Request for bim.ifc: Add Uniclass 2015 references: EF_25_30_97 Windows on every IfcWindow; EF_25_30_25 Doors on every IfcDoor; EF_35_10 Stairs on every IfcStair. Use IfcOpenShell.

First a look at what the model holds.

```python
import ifcopenshell

model = ifcopenshell.open("bim.ifc")
print(model.schema)
print("classifications:", [c.Name for c in model.by_type("IfcClassification")])
for ifc_class in ("IfcDoor", "IfcRoof", "IfcStair", "IfcWall", "IfcWindow"):
    print(ifc_class, len(model.by_type(ifc_class)))
```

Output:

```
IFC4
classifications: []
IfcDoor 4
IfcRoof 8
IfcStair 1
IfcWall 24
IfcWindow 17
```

```python
import ifcopenshell
import ifcopenshell.api.classification

model = ifcopenshell.open("bim.ifc")

system = ifcopenshell.api.classification.add_classification(model, classification="Uniclass 2015")

codes = {
    "IfcWindow": ("EF_25_30_97", "Windows"),
    "IfcDoor": ("EF_25_30_25", "Doors"),
    "IfcStair": ("EF_35_10", "Stairs"),
}
for ifc_class, (code, name) in codes.items():
    products = model.by_type(ifc_class)
    ifcopenshell.api.classification.add_reference(
        model, products=products, classification=system, identification=code, name=name
    )
    print(code, len(products))

model.write("bim_rev.ifc")
```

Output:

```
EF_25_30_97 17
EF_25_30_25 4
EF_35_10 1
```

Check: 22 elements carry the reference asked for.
